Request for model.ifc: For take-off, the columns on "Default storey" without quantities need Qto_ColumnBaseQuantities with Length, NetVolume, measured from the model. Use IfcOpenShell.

First a look at what the model holds.

```python
import ifcopenshell
import ifcopenshell.util.element
import ifcopenshell.util.unit

model = ifcopenshell.open("model.ifc")
print(model.schema)
for unit_type in ("LENGTHUNIT", "AREAUNIT", "VOLUMEUNIT"):
    print(unit_type, ifcopenshell.util.unit.calculate_unit_scale(model, unit_type))
storey = next(s for s in model.by_type("IfcBuildingStorey") if s.Name == "Default storey")
columns = [e for e in ifcopenshell.util.element.get_decomposition(storey) if e.is_a("IfcColumn")]
for e in sorted(columns, key=lambda e: e.id()):
    print(e.id(), e.is_a(), e.Name, list(ifcopenshell.util.element.get_psets(e, qtos_only=True)), sep=" | ")
```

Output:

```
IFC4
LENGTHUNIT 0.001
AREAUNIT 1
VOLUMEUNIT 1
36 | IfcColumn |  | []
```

```python
import ifcopenshell
import ifcopenshell.api.pset
import ifcopenshell.geom
import ifcopenshell.util.element
import ifcopenshell.util.shape
import ifcopenshell.util.unit

model = ifcopenshell.open("model.ifc")
unit_scale = ifcopenshell.util.unit.calculate_unit_scale(model)
volume_scale = ifcopenshell.util.unit.calculate_unit_scale(model, "VOLUMEUNIT")
settings = ifcopenshell.geom.settings()

storey = next(s for s in model.by_type("IfcBuildingStorey") if s.Name == "Default storey")
columns = [e for e in ifcopenshell.util.element.get_decomposition(storey) if e.is_a("IfcColumn")]

for e in sorted(columns, key=lambda e: e.id()):
    if ifcopenshell.util.element.get_psets(e, qtos_only=True, should_inherit=False):
        continue
    # Geometry comes back in metres, in the element's own axes.
    shape = ifcopenshell.geom.create_shape(settings, e)
    values = {
        "Length": ifcopenshell.util.shape.get_z(shape.geometry) / unit_scale,
        "NetVolume": ifcopenshell.util.shape.get_volume(shape.geometry) / volume_scale,
    }
    qto = ifcopenshell.api.pset.add_qto(model, product=e, name="Qto_ColumnBaseQuantities")
    ifcopenshell.api.pset.edit_qto(model, qto=qto, properties=values)
    print(e.id(), {k: round(v, 3) for k, v in values.items()})

model.write("model_updated.ifc")
```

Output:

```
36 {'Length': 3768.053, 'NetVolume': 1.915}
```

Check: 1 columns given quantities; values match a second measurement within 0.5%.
